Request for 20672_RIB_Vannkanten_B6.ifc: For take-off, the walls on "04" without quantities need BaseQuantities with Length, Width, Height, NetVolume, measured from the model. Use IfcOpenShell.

First a look at what the model holds.

```python
import ifcopenshell
import ifcopenshell.util.element
import ifcopenshell.util.unit

model = ifcopenshell.open("20672_RIB_Vannkanten_B6.ifc")
print(model.schema)
for unit_type in ("LENGTHUNIT", "AREAUNIT", "VOLUMEUNIT"):
    print(unit_type, ifcopenshell.util.unit.calculate_unit_scale(model, unit_type))
storey = next(s for s in model.by_type("IfcBuildingStorey") if s.Name == "04")
walls = [e for e in ifcopenshell.util.element.get_decomposition(storey) if e.is_a("IfcWall")]
for e in sorted(walls, key=lambda e: e.id()):
    print(e.id(), e.is_a(), e.Name, list(ifcopenshell.util.element.get_psets(e, qtos_only=True)), sep=" | ")
```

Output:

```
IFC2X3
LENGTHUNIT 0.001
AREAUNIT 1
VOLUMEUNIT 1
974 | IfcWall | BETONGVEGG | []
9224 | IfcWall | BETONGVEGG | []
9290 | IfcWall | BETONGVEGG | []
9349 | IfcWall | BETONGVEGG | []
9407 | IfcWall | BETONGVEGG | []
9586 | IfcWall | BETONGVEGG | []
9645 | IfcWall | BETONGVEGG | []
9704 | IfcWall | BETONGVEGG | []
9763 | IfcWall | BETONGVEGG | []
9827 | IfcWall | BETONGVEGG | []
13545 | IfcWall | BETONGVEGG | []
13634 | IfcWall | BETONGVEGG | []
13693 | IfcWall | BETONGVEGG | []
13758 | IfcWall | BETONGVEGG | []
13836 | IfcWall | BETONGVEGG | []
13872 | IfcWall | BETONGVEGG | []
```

```python
import ifcopenshell
import ifcopenshell.api.pset
import ifcopenshell.geom
import ifcopenshell.util.element
import ifcopenshell.util.shape
import ifcopenshell.util.unit

model = ifcopenshell.open("20672_RIB_Vannkanten_B6.ifc")
unit_scale = ifcopenshell.util.unit.calculate_unit_scale(model)
volume_scale = ifcopenshell.util.unit.calculate_unit_scale(model, "VOLUMEUNIT")
settings = ifcopenshell.geom.settings()

storey = next(s for s in model.by_type("IfcBuildingStorey") if s.Name == "04")
walls = [e for e in ifcopenshell.util.element.get_decomposition(storey) if e.is_a("IfcWall")]

for e in sorted(walls, key=lambda e: e.id()):
    if ifcopenshell.util.element.get_psets(e, qtos_only=True, should_inherit=False):
        continue
    # Geometry comes back in metres, in the element's own axes.
    shape = ifcopenshell.geom.create_shape(settings, e)
    values = {
        "Length": ifcopenshell.util.shape.get_x(shape.geometry) / unit_scale,
        "Width": ifcopenshell.util.shape.get_y(shape.geometry) / unit_scale,
        "Height": ifcopenshell.util.shape.get_z(shape.geometry) / unit_scale,
        "NetVolume": ifcopenshell.util.shape.get_volume(shape.geometry) / volume_scale,
    }
    qto = ifcopenshell.api.pset.add_qto(model, product=e, name="BaseQuantities")
    ifcopenshell.api.pset.edit_qto(model, qto=qto, properties=values)
    print(e.id(), {k: round(v, 3) for k, v in values.items()})

model.write("20672_RIB_Vannkanten_B6_rev.ifc")
```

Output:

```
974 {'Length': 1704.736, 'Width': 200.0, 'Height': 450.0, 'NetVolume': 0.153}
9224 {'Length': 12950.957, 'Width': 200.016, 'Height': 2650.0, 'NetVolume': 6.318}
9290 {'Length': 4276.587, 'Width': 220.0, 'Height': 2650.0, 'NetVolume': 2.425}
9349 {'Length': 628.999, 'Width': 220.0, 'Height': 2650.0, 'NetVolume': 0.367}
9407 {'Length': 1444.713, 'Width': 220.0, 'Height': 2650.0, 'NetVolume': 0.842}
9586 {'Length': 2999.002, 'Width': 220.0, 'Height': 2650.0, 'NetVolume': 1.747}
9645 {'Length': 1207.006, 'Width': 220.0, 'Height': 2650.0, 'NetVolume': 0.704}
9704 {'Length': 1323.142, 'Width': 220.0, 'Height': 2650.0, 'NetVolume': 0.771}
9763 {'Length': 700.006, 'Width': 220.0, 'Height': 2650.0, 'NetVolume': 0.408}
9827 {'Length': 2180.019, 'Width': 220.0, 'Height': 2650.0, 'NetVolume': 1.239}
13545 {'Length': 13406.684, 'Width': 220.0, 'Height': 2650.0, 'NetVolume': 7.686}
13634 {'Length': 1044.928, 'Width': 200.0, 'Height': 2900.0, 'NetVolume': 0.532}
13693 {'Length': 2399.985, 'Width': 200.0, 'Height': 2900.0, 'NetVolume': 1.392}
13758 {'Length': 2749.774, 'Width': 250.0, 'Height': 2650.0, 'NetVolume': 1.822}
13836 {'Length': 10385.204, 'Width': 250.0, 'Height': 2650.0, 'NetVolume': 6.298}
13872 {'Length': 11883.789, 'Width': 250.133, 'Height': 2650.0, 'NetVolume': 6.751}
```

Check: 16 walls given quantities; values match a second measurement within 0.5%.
